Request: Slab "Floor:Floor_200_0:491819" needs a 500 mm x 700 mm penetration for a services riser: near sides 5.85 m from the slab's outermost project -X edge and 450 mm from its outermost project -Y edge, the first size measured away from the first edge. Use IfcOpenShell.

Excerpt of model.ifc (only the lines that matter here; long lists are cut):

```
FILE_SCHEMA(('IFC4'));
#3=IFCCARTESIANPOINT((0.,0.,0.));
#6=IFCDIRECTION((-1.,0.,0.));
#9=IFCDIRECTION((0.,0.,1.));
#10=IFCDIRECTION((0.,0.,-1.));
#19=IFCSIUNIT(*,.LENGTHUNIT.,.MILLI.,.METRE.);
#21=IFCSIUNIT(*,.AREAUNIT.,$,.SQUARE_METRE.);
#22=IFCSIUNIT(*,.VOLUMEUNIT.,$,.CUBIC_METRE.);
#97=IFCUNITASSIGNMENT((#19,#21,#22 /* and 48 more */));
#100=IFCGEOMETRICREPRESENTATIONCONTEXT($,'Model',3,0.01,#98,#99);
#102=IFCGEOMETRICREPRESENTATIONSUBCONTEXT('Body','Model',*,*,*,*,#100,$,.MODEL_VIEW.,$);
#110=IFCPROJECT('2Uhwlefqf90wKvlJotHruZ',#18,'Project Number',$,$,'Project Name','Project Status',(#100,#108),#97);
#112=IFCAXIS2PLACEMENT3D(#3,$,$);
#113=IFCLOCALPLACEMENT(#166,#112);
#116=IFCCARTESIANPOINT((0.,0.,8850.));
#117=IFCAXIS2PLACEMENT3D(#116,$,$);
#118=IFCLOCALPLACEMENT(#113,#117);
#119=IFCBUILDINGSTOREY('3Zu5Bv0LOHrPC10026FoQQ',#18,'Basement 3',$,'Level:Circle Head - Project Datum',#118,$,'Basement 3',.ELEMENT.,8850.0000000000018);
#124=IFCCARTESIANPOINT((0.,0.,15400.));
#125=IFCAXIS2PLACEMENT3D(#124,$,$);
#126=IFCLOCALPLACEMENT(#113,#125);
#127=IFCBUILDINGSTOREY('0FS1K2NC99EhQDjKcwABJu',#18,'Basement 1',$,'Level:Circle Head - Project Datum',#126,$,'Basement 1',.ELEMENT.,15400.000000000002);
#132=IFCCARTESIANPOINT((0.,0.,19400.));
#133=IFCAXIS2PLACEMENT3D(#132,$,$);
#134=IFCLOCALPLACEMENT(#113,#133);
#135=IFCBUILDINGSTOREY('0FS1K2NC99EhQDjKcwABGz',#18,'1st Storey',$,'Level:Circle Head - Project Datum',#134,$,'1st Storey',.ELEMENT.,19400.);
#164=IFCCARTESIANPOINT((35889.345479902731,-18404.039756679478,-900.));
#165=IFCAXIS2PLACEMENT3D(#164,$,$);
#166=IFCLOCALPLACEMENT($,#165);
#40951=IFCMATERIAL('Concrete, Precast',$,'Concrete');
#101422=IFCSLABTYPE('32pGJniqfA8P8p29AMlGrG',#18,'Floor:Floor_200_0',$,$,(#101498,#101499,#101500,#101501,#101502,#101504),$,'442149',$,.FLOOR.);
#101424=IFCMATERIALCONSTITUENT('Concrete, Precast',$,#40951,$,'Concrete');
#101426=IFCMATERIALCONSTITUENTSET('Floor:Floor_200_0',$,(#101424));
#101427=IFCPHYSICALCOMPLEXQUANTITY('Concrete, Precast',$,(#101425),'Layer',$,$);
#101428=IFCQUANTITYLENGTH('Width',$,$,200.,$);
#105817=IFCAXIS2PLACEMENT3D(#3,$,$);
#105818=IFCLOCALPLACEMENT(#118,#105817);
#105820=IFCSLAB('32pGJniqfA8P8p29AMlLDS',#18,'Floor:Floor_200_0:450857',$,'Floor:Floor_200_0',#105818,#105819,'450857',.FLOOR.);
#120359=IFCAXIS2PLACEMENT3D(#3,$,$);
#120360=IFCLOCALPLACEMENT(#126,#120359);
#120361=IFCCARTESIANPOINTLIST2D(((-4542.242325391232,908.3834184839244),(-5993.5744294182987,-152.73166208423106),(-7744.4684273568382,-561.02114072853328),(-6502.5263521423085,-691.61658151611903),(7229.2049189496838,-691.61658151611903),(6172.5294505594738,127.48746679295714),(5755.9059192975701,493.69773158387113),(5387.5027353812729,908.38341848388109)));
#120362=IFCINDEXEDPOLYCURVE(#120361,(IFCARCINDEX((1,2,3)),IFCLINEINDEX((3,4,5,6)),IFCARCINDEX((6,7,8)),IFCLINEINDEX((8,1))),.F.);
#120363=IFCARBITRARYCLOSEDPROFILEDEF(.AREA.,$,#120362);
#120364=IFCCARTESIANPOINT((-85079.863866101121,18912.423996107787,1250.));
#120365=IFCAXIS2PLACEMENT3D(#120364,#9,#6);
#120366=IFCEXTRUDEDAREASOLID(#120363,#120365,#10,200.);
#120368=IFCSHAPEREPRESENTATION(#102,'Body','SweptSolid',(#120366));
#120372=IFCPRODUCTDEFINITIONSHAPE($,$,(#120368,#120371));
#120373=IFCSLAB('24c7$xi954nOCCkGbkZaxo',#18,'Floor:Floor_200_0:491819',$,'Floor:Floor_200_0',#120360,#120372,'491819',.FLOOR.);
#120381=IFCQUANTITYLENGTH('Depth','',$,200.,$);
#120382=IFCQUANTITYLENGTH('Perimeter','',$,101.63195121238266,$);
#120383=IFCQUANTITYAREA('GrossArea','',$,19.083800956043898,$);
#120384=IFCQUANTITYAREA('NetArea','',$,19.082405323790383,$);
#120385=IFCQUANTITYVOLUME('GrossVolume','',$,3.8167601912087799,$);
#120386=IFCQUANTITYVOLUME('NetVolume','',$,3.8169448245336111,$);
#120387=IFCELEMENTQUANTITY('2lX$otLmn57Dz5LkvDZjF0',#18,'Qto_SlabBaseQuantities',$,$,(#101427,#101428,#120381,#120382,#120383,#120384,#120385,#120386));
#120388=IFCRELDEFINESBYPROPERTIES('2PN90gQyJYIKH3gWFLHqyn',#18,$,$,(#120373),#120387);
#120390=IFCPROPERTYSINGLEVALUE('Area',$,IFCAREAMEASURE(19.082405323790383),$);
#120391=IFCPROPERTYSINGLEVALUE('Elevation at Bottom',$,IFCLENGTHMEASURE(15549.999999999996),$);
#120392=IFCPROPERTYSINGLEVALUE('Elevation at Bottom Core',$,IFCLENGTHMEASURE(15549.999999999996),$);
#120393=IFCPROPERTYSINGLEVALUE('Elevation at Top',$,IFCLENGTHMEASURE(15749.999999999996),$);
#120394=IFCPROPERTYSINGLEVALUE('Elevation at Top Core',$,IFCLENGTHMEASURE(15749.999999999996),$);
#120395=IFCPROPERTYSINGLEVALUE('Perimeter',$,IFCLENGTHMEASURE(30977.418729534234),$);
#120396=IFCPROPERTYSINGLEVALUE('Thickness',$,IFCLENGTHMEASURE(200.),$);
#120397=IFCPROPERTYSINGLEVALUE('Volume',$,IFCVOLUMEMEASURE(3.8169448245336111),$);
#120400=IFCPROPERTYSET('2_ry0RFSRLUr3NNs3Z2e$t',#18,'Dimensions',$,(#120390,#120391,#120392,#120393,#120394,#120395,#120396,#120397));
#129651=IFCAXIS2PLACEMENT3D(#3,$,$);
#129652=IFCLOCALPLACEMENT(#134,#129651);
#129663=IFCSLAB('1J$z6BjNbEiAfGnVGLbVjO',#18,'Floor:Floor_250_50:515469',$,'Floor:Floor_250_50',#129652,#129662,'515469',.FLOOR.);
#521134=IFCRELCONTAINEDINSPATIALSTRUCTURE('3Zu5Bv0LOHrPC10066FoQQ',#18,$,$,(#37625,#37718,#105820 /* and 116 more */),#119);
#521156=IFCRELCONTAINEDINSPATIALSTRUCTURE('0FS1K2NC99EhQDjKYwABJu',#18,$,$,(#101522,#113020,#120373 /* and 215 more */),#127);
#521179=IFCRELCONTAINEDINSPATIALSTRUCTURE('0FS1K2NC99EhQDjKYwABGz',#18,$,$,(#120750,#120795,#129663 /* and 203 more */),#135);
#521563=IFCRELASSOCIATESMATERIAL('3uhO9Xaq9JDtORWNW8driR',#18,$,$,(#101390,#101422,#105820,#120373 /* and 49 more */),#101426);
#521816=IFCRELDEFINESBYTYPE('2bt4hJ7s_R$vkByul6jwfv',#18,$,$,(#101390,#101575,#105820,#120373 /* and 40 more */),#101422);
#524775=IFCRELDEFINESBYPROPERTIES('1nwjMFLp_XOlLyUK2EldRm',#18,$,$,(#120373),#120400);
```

```python
import numpy as np
import ifcopenshell
import ifcopenshell.api.feature
import ifcopenshell.api.geometry
import ifcopenshell.api.pset
import ifcopenshell.api.root
import ifcopenshell.geom
import ifcopenshell.util.element
import ifcopenshell.util.placement
import ifcopenshell.util.representation
import ifcopenshell.util.shape
import ifcopenshell.util.unit

model = ifcopenshell.open("model.ifc")
unit_scale = ifcopenshell.util.unit.calculate_unit_scale(model)
area_scale = ifcopenshell.util.unit.calculate_unit_scale(model, "AREAUNIT")
volume_scale = ifcopenshell.util.unit.calculate_unit_scale(model, "VOLUMEUNIT")
settings = ifcopenshell.geom.settings()


def volume(element):
    """Net volume in cubic metres, openings subtracted."""
    shape = ifcopenshell.geom.create_shape(settings, element)
    return ifcopenshell.util.shape.get_volume(shape.geometry)


slab = model.by_guid("24c7$xi954nOCCkGbkZaxo")
before = volume(slab)

# Extent in the slab's own axes, in metres. The edges named are its -X and -Y sides.
slab_shape = ifcopenshell.geom.create_shape(settings, slab)
vertices = ifcopenshell.util.shape.get_vertices(slab_shape.geometry)
x_min, y_min, bottom = vertices.min(axis=0)
top = vertices[:, 2].max()

opening = ifcopenshell.api.root.create_entity(model, ifc_class="IfcOpeningElement", name="Services riser opening", predefined_type="OPENING")
context = ifcopenshell.util.representation.get_context(model, "Model", "Body", "MODEL_VIEW")
width, depth = 0.5, 0.7
outline = [(0.0, 0.0), (width, 0.0), (width, depth), (0.0, depth), (0.0, 0.0)]
# Overshoot both faces by 50 mm so the cut is clean.
shape = ifcopenshell.api.geometry.add_slab_representation(
    model, context=context, depth=top - bottom + 0.1, polyline=outline
)
ifcopenshell.api.geometry.assign_representation(model, product=opening, representation=shape)

matrix = ifcopenshell.util.placement.get_local_placement(slab.ObjectPlacement)
matrix[:, 3] = matrix @ np.append(np.array([x_min + 5.85, y_min + 0.45, bottom - 0.05]) / unit_scale, 1.0)
ifcopenshell.api.geometry.edit_object_placement(model, product=opening, matrix=matrix, is_si=False)
ifcopenshell.api.feature.add_feature(model, feature=opening, element=slab)

after = volume(slab)

# Update the slab's stored quantities.
qto = model.by_id(ifcopenshell.util.element.get_pset(slab, "Qto_SlabBaseQuantities", should_inherit=False)["id"])
ifcopenshell.api.pset.edit_qto(model, qto=qto, properties={
    "NetArea": after / (top - bottom) / area_scale,
    "NetVolume": after / volume_scale,
})
pset = model.by_id(ifcopenshell.util.element.get_pset(slab, "Dimensions", should_inherit=False)["id"])
ifcopenshell.api.pset.edit_pset(model, pset=pset, properties={
    "Area": model.create_entity("IfcAreaMeasure", after / (top - bottom) / area_scale),
    "Volume": model.create_entity("IfcVolumeMeasure", after / volume_scale),
})

print(f"slab volume {before:.3f} -> {after:.3f} m3")

model.write("model_updated.ifc")
```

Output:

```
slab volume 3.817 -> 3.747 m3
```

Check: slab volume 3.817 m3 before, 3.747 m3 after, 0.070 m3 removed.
